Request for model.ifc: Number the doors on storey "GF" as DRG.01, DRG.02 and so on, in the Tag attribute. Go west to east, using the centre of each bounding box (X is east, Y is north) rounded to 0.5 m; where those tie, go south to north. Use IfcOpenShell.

First a look at what the model holds.

```python
import ifcopenshell
import ifcopenshell.util.element
import ifcopenshell.util.placement

model = ifcopenshell.open("model.ifc")
print(model.schema)
storey = next(s for s in model.by_type("IfcBuildingStorey") if s.Name == "GF")
doors = [e for e in ifcopenshell.util.element.get_decomposition(storey) if e.is_a("IfcDoor")]
for e in sorted(doors, key=lambda e: e.id()):
    origin = ifcopenshell.util.placement.get_local_placement(e.ObjectPlacement)[:3, 3]
    print(e.id(), e.Tag, e.Name, origin.round(2) + 0.0, sep=" | ")
```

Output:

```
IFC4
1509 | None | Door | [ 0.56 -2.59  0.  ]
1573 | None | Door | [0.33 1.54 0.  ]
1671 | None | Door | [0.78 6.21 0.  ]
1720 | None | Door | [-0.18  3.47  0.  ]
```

```python
import ifcopenshell
import ifcopenshell.geom
import ifcopenshell.util.element
import ifcopenshell.util.shape

model = ifcopenshell.open("model.ifc")
settings = ifcopenshell.geom.settings()
settings.set("use-world-coords", True)


def centre(element):
    shape = ifcopenshell.geom.create_shape(settings, element)
    return ifcopenshell.util.shape.get_bbox_centroid(shape.geometry)


storey = next(s for s in model.by_type("IfcBuildingStorey") if s.Name == "GF")
doors = [e for e in ifcopenshell.util.element.get_decomposition(storey) if e.is_a("IfcDoor")]

# Insertion points can sit at a corner or the storey origin, so sort by the geometry (in metres).
centres = {e: centre(e) for e in doors}
doors.sort(key=lambda e: (round(centres[e][0] / 0.5), centres[e][1]))

for i, e in enumerate(doors, start=1):
    number = f"DRG.{i:02d}"
    e.Tag = number
    print(e.id(), number)

model.write("model_updated.ifc")
```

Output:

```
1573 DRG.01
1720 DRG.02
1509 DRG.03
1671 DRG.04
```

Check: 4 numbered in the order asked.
